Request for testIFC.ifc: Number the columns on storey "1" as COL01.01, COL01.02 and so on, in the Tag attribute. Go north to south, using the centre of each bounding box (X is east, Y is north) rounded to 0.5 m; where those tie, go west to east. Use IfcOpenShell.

First a look at what the model holds.

```python
import ifcopenshell
import ifcopenshell.util.element
import ifcopenshell.util.placement

model = ifcopenshell.open("testIFC.ifc")
print(model.schema)
storey = next(s for s in model.by_type("IfcBuildingStorey") if s.Name == "1")
columns = [e for e in ifcopenshell.util.element.get_decomposition(storey) if e.is_a("IfcColumn")]
for e in sorted(columns, key=lambda e: e.id()):
    origin = ifcopenshell.util.placement.get_local_placement(e.ObjectPlacement)[:3, 3]
    print(e.id(), e.Tag, e.Name, origin.round(2) + 0.0, sep=" | ")
```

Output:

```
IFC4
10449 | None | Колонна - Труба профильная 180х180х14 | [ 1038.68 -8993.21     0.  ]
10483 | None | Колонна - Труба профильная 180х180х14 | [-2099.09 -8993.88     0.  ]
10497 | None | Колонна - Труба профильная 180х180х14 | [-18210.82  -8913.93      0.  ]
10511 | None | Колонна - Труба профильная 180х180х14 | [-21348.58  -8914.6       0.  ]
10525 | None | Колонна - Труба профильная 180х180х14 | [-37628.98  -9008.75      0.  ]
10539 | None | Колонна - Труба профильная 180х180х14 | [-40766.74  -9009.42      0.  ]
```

```python
import ifcopenshell
import ifcopenshell.geom
import ifcopenshell.util.element
import ifcopenshell.util.shape

model = ifcopenshell.open("testIFC.ifc")
settings = ifcopenshell.geom.settings()
settings.set("use-world-coords", True)


def centre(element):
    shape = ifcopenshell.geom.create_shape(settings, element)
    return ifcopenshell.util.shape.get_bbox_centroid(shape.geometry)


storey = next(s for s in model.by_type("IfcBuildingStorey") if s.Name == "1")
columns = [e for e in ifcopenshell.util.element.get_decomposition(storey) if e.is_a("IfcColumn")]

# Insertion points can sit at a corner or the storey origin, so sort by the geometry (in metres).
centres = {e: centre(e) for e in columns}
columns.sort(key=lambda e: (-round(centres[e][1] / 0.5), centres[e][0]))

for i, e in enumerate(columns, start=1):
    number = f"COL01.{i:02d}"
    e.Tag = number
    print(e.id(), number)

model.write("testIFC_v2.ifc")
```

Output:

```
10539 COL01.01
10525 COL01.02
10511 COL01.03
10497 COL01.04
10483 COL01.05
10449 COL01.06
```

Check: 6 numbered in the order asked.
